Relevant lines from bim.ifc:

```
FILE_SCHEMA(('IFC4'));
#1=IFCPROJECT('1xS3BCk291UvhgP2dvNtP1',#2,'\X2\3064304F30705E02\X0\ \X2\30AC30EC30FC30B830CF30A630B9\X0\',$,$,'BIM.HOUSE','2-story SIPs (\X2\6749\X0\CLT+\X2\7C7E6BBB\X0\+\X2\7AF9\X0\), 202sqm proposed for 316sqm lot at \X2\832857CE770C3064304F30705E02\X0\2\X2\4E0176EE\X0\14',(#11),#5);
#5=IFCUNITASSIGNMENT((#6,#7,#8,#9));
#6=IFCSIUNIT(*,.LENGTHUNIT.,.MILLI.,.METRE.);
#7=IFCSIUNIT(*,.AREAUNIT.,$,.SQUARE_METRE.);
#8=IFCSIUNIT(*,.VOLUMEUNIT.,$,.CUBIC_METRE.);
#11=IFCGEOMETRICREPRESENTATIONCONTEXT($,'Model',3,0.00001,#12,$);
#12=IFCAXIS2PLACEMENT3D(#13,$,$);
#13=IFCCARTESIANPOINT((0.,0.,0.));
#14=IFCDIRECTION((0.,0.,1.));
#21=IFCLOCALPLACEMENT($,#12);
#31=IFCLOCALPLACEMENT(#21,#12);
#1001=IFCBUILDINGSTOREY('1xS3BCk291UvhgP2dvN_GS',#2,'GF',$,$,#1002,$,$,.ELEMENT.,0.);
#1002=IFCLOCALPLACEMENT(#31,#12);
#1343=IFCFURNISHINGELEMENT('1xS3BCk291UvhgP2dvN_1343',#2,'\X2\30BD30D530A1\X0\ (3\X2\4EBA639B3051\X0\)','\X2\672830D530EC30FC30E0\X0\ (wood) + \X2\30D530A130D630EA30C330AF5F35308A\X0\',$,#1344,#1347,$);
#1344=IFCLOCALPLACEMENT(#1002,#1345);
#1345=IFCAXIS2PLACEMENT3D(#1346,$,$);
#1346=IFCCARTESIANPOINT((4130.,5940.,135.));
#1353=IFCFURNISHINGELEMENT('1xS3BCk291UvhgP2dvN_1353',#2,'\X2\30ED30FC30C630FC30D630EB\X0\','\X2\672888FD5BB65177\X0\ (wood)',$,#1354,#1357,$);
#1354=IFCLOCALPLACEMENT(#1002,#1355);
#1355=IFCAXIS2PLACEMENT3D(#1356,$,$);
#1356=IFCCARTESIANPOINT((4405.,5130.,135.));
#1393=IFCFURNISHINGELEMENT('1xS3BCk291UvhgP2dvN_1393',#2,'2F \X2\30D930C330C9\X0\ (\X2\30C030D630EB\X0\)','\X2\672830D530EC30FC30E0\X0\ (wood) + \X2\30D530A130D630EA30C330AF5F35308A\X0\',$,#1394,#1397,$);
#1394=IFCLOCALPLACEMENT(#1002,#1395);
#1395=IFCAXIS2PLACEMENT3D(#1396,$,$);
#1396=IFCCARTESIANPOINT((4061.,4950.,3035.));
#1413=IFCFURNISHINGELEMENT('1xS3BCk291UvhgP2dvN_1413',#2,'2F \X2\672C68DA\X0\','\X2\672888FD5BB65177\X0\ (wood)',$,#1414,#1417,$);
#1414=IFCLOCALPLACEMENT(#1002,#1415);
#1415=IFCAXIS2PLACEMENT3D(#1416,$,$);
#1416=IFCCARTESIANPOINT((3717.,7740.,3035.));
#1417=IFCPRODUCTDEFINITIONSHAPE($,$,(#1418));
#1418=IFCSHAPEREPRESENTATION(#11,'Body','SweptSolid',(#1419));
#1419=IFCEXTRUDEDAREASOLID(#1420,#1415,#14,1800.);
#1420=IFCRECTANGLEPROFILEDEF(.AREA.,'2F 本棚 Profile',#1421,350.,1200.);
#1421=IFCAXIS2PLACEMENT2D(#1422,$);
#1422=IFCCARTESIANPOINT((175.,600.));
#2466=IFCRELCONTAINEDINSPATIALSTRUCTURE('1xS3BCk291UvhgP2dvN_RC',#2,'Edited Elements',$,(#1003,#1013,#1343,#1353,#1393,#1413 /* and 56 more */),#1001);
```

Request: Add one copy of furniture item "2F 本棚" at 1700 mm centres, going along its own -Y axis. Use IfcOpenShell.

```python
import ifcopenshell
import ifcopenshell.api.geometry
import ifcopenshell.api.root
import ifcopenshell.util.element
import ifcopenshell.util.placement
import ifcopenshell.util.unit

model = ifcopenshell.open("bim.ifc")
unit_scale = ifcopenshell.util.unit.calculate_unit_scale(model)


def reuse_history(source, copy):
    """copy_class also copies each property set's owner history, people and application; keep the originals."""
    for rel in copy.IsDefinedBy:
        if rel.is_a("IfcRelDefinesByProperties") and (history := rel.RelatingPropertyDefinition.OwnerHistory):
            rel.RelatingPropertyDefinition.OwnerHistory = source.OwnerHistory
            ifcopenshell.util.element.remove_deep2(model, history)


source = model.by_guid("1xS3BCk291UvhgP2dvN_1413")
base = ifcopenshell.util.placement.get_local_placement(source.ObjectPlacement)
step = -base[:3, 1] * 1.7 / unit_scale

for i in range(1, 2):
    copy = ifcopenshell.api.root.copy_class(model, product=source)
    copy.Representation = ifcopenshell.util.element.copy_deep(
        model, source.Representation, exclude=["IfcGeometricRepresentationContext", "IfcRepresentationMap"]
    )
    reuse_history(source, copy)
    matrix = base.copy()
    matrix[:3, 3] += i * step
    print("added at", matrix[:3, 3].round(3) + 0.0)
    ifcopenshell.api.geometry.edit_object_placement(model, product=copy, matrix=matrix, is_si=False)

model.write("bim_v2.ifc")
```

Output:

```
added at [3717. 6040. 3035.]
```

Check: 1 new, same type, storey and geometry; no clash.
